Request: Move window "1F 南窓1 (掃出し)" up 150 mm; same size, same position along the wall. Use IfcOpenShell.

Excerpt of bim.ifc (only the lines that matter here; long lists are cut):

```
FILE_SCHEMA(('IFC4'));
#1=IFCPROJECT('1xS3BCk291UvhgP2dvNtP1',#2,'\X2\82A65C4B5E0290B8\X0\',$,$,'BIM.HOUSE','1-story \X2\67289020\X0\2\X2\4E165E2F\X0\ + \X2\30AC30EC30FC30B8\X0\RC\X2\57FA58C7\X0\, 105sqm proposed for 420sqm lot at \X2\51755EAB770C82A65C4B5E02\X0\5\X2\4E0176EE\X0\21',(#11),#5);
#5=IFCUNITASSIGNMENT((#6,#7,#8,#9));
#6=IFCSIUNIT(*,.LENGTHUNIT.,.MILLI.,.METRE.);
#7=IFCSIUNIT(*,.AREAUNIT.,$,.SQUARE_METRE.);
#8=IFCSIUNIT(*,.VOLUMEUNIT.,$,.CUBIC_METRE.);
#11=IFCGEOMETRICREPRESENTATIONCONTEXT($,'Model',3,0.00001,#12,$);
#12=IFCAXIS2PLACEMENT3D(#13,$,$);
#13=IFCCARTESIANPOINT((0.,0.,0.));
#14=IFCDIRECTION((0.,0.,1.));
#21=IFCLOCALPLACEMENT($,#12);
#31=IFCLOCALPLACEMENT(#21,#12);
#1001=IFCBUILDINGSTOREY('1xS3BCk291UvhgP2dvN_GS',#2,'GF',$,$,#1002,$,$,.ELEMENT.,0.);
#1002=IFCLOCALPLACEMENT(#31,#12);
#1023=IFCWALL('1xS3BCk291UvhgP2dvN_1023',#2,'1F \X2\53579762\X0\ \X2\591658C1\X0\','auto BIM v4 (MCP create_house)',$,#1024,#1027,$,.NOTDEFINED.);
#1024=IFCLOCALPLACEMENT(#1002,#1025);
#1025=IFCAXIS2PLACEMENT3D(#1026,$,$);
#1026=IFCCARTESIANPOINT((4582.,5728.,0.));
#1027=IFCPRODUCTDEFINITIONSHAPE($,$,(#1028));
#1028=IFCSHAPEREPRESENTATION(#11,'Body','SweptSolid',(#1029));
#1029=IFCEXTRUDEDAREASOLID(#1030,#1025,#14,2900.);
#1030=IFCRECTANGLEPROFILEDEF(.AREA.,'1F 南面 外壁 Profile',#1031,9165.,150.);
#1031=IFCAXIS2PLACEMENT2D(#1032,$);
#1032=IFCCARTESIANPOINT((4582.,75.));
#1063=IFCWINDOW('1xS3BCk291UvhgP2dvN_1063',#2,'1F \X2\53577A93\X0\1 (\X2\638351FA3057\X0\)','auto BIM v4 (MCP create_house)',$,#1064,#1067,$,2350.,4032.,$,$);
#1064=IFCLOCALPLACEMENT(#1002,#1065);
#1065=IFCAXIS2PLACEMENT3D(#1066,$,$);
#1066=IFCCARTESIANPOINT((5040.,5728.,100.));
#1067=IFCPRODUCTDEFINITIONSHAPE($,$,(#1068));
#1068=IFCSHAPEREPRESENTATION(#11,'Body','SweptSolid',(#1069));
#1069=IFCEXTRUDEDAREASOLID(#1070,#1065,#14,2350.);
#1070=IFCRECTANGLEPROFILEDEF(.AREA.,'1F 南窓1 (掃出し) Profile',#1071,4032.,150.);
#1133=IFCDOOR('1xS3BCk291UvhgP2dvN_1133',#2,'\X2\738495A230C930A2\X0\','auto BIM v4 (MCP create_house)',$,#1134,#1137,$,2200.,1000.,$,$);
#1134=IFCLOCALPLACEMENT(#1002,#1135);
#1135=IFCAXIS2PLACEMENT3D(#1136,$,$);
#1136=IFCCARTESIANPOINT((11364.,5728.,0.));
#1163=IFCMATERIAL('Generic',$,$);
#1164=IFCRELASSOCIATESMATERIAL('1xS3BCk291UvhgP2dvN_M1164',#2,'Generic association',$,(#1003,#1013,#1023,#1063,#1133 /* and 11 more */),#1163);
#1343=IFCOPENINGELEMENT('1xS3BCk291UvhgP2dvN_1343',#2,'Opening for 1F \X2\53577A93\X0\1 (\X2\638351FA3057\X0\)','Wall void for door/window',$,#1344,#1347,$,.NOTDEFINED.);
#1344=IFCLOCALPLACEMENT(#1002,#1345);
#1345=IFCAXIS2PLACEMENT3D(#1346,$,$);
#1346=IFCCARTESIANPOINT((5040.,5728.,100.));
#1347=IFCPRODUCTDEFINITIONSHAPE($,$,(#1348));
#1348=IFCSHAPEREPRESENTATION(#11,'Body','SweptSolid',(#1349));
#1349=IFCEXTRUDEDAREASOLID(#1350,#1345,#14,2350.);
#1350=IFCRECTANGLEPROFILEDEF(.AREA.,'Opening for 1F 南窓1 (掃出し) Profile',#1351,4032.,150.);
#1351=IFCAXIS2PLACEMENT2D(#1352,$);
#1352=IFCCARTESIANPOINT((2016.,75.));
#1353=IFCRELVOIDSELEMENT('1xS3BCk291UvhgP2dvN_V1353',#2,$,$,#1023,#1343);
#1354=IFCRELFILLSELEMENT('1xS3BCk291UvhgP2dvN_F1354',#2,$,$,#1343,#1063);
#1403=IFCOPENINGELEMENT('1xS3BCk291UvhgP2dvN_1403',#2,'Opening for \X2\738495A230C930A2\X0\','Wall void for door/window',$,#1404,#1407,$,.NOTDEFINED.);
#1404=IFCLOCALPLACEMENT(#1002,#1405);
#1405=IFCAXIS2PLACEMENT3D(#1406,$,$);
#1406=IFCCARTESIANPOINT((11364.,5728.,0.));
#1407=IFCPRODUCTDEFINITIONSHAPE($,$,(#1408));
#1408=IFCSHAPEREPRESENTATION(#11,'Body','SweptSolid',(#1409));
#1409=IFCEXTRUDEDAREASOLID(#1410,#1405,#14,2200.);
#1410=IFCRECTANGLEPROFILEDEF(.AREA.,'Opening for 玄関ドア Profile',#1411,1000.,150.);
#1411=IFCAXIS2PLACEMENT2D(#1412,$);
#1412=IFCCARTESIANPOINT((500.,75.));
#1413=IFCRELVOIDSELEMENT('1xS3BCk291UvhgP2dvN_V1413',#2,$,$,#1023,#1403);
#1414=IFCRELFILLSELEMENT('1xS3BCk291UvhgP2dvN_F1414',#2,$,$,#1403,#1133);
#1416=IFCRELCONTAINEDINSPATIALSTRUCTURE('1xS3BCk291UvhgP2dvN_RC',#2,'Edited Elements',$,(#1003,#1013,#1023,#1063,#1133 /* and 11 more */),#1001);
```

```python
import numpy as np
import ifcopenshell
import ifcopenshell.api.geometry
import ifcopenshell.util.placement
import ifcopenshell.util.unit

model = ifcopenshell.open("bim.ifc")
unit_scale = ifcopenshell.util.unit.calculate_unit_scale(model)

window = model.by_guid("1xS3BCk291UvhgP2dvN_1063")
opening = window.FillsVoids[0].RelatingOpeningElement
dz = 0.15 / unit_scale

shift = np.array([0.0, 0.0, dz])
# The window is not placed relative to its opening, so move both.
for product in (opening, window):
    matrix = ifcopenshell.util.placement.get_local_placement(product.ObjectPlacement)
    matrix[:3, 3] += shift
    ifcopenshell.api.geometry.edit_object_placement(model, product=product, matrix=matrix, is_si=False)

print(f"moved by {dz * unit_scale:+.3f} m")

model.write("bim_edited.ifc")
```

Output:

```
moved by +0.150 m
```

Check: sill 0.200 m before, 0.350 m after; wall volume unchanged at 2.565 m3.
